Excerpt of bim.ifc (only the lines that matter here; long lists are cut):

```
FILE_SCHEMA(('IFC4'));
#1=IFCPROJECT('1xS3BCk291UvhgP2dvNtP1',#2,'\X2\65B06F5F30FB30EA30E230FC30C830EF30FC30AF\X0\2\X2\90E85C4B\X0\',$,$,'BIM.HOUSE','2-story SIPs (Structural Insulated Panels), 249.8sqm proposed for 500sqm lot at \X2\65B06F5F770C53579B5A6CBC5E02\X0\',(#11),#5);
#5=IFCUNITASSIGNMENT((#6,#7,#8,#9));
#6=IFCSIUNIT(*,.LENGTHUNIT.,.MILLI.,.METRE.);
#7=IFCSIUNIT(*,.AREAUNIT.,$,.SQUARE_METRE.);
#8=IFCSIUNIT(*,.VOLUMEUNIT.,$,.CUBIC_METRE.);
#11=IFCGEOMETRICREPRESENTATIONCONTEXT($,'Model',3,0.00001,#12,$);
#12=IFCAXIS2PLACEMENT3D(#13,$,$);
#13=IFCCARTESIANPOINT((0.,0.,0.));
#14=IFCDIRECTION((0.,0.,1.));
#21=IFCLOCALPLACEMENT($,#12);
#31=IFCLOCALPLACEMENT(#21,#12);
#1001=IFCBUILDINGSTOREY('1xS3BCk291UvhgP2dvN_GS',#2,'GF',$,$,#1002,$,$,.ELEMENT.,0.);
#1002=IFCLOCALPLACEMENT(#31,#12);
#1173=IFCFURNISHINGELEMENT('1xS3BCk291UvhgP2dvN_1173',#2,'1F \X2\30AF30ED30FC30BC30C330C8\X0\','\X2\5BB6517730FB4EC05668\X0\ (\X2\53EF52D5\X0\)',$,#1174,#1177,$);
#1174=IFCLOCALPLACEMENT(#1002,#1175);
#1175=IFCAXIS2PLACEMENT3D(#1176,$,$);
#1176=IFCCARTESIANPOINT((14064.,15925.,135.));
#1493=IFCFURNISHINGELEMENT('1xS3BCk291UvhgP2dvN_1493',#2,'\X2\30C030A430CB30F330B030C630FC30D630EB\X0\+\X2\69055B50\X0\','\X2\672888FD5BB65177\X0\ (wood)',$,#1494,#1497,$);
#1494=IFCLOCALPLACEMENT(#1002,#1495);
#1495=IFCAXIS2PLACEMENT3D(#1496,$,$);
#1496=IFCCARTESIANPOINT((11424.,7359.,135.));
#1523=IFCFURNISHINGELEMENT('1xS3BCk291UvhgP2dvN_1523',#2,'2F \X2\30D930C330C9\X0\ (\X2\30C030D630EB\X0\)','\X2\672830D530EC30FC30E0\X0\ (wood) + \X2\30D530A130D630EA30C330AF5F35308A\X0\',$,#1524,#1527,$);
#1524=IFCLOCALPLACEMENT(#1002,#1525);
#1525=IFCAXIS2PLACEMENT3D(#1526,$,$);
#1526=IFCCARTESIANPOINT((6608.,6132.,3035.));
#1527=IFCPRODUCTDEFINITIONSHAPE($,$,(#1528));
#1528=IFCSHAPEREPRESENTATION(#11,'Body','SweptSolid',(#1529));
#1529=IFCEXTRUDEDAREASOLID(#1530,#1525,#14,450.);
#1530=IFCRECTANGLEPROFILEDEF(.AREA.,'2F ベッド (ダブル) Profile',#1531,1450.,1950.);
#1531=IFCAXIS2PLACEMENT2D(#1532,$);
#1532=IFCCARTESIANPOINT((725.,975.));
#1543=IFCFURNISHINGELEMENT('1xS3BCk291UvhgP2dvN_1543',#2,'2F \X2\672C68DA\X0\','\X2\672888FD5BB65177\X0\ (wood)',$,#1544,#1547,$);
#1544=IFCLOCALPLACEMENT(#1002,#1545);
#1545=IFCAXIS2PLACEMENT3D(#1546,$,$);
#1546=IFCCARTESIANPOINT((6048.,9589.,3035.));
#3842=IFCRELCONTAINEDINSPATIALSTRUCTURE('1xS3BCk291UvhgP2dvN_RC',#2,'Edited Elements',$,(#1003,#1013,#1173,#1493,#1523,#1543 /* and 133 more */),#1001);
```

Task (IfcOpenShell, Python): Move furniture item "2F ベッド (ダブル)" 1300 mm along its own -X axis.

```python
import ifcopenshell
import ifcopenshell.api.geometry
import ifcopenshell.util.placement
import ifcopenshell.util.unit

model = ifcopenshell.open("bim.ifc")
unit_scale = ifcopenshell.util.unit.calculate_unit_scale(model)

item = model.by_guid("1xS3BCk291UvhgP2dvN_1523")
matrix = ifcopenshell.util.placement.get_local_placement(item.ObjectPlacement)
matrix[:3, 3] -= matrix[:3, 0] * 1.3 / unit_scale
ifcopenshell.api.geometry.edit_object_placement(model, product=item, matrix=matrix, is_si=False)

print(ifcopenshell.util.placement.get_local_placement(item.ObjectPlacement).round(3) + 0.0)

model.write("bim_rev.ifc")
```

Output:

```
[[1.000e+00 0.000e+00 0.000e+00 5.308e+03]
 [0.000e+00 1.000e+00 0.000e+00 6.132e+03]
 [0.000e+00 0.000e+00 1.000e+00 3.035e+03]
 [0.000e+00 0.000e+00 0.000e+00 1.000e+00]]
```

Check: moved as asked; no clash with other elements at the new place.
